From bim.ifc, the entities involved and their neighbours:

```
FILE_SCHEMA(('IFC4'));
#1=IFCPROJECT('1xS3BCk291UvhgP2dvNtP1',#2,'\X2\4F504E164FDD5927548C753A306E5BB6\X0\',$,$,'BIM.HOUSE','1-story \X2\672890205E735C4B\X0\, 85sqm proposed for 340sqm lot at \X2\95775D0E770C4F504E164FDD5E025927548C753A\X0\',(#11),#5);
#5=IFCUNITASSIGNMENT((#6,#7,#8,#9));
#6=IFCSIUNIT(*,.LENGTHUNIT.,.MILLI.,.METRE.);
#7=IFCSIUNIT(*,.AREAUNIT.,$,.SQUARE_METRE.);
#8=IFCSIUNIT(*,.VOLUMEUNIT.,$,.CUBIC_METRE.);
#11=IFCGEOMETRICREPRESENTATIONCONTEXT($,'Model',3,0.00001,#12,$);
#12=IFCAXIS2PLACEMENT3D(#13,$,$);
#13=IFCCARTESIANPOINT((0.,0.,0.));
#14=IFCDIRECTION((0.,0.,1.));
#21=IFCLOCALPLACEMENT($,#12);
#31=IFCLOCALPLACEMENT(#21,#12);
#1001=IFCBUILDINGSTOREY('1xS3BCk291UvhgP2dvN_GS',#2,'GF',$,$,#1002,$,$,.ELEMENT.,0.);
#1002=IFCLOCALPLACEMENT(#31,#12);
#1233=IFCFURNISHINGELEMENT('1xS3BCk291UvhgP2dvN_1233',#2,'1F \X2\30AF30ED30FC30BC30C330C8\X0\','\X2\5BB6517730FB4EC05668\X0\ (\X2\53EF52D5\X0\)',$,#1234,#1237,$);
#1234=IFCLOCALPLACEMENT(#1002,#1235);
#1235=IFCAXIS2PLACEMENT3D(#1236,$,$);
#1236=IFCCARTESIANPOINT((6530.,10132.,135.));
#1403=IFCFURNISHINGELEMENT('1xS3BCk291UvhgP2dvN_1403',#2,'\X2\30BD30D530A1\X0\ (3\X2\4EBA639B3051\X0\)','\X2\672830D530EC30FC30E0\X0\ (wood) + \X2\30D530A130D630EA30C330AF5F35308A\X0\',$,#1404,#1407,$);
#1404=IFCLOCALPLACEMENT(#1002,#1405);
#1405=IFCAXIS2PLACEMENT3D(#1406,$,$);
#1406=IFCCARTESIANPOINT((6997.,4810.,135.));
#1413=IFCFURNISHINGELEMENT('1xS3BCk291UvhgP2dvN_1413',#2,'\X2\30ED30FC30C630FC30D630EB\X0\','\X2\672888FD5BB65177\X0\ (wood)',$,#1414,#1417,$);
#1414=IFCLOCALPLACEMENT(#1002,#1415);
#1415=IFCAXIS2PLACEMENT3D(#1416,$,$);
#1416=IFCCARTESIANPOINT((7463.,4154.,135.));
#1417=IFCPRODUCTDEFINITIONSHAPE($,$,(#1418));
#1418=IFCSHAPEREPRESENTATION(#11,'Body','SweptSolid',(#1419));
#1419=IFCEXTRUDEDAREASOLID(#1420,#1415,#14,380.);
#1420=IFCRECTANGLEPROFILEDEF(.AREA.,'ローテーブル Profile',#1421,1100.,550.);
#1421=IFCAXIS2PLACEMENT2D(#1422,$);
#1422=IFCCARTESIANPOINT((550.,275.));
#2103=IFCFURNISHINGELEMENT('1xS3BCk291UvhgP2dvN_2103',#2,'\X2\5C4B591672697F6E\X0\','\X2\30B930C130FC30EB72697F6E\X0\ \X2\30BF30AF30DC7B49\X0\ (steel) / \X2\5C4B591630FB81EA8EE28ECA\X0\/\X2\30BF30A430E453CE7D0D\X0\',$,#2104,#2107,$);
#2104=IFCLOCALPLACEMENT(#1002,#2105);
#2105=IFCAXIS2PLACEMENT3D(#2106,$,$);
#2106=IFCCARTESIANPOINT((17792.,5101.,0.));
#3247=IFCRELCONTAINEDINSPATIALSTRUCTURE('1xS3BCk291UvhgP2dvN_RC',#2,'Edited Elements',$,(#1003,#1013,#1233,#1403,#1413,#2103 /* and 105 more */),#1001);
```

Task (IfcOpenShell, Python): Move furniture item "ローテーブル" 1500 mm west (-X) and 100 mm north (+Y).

```python
import ifcopenshell
import ifcopenshell.api.geometry
import ifcopenshell.util.placement
import ifcopenshell.util.unit

model = ifcopenshell.open("bim.ifc")
unit_scale = ifcopenshell.util.unit.calculate_unit_scale(model)

item = model.by_id(1413)
matrix = ifcopenshell.util.placement.get_local_placement(item.ObjectPlacement)
matrix[0, 3] -= 1.5 / unit_scale
matrix[1, 3] += 0.1 / unit_scale
ifcopenshell.api.geometry.edit_object_placement(model, product=item, matrix=matrix, is_si=False)

print(ifcopenshell.util.placement.get_local_placement(item.ObjectPlacement).round(3) + 0.0)

model.write("bim_rev.ifc")
```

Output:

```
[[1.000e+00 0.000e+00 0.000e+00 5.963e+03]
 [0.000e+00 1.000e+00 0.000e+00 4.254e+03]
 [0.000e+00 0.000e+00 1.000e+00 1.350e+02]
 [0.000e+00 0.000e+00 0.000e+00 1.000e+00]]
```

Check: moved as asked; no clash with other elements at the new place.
